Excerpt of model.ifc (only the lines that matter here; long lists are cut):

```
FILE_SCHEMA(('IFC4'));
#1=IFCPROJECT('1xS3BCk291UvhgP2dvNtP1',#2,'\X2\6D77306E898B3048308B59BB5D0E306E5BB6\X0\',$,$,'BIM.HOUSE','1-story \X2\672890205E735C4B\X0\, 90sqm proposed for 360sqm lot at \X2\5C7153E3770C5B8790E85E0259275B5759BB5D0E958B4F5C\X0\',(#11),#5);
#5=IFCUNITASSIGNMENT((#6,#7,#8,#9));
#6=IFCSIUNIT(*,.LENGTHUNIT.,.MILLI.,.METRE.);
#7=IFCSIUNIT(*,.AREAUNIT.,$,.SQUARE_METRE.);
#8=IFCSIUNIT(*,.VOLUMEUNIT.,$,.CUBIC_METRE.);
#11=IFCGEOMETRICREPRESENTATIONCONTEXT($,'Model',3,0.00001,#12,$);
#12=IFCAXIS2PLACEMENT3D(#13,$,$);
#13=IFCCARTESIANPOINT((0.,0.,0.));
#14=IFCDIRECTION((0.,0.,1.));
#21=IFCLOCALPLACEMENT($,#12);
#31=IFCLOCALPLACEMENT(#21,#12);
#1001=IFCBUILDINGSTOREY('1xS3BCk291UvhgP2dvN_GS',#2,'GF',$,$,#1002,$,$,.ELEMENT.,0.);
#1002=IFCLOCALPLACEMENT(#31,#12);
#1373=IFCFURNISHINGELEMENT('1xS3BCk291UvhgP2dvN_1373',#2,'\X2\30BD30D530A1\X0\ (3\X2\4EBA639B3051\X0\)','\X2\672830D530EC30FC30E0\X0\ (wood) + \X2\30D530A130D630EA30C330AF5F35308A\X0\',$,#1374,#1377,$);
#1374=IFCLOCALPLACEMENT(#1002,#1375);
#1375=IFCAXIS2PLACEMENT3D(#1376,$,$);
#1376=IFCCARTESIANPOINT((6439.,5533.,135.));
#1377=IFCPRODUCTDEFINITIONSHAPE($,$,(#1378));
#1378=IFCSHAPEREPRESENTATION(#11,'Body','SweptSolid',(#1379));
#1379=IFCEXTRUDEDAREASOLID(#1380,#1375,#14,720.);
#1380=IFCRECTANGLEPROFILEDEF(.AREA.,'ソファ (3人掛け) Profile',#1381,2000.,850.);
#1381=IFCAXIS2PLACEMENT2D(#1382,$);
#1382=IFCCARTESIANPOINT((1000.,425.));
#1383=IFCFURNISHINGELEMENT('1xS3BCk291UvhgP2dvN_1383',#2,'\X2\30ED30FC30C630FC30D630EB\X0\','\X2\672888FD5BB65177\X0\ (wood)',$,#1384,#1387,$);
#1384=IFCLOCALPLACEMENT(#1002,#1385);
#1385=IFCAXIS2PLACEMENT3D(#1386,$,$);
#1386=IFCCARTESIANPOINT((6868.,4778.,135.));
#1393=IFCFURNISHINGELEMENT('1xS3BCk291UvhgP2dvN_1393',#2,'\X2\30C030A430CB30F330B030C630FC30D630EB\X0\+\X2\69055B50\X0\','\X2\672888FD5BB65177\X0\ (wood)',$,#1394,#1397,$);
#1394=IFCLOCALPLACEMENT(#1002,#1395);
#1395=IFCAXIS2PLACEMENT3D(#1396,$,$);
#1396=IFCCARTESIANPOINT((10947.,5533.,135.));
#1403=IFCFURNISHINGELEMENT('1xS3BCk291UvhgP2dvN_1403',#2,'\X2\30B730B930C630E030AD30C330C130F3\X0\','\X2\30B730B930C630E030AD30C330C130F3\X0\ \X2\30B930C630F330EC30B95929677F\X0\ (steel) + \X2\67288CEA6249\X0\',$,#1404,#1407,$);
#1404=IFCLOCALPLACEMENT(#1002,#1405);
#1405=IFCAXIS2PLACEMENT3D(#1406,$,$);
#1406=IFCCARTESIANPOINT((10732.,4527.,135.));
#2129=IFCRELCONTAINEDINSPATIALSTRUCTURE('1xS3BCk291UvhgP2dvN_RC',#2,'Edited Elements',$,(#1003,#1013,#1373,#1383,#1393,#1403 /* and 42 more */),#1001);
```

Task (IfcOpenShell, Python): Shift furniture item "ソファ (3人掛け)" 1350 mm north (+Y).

```python
import ifcopenshell
import ifcopenshell.api.geometry
import ifcopenshell.util.placement

model = ifcopenshell.open("model.ifc")

item = model.by_id(1373)
matrix = ifcopenshell.util.placement.get_local_placement(item.ObjectPlacement)
matrix[1, 3] += 1350.0
ifcopenshell.api.geometry.edit_object_placement(model, product=item, matrix=matrix, is_si=False)

print(ifcopenshell.util.placement.get_local_placement(item.ObjectPlacement).round(3) + 0.0)

model.write("model-out.ifc")
```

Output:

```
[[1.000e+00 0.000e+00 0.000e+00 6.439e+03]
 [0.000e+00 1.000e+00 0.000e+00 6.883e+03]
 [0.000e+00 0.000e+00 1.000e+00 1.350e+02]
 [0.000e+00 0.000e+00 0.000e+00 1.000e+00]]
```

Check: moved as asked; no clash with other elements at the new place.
